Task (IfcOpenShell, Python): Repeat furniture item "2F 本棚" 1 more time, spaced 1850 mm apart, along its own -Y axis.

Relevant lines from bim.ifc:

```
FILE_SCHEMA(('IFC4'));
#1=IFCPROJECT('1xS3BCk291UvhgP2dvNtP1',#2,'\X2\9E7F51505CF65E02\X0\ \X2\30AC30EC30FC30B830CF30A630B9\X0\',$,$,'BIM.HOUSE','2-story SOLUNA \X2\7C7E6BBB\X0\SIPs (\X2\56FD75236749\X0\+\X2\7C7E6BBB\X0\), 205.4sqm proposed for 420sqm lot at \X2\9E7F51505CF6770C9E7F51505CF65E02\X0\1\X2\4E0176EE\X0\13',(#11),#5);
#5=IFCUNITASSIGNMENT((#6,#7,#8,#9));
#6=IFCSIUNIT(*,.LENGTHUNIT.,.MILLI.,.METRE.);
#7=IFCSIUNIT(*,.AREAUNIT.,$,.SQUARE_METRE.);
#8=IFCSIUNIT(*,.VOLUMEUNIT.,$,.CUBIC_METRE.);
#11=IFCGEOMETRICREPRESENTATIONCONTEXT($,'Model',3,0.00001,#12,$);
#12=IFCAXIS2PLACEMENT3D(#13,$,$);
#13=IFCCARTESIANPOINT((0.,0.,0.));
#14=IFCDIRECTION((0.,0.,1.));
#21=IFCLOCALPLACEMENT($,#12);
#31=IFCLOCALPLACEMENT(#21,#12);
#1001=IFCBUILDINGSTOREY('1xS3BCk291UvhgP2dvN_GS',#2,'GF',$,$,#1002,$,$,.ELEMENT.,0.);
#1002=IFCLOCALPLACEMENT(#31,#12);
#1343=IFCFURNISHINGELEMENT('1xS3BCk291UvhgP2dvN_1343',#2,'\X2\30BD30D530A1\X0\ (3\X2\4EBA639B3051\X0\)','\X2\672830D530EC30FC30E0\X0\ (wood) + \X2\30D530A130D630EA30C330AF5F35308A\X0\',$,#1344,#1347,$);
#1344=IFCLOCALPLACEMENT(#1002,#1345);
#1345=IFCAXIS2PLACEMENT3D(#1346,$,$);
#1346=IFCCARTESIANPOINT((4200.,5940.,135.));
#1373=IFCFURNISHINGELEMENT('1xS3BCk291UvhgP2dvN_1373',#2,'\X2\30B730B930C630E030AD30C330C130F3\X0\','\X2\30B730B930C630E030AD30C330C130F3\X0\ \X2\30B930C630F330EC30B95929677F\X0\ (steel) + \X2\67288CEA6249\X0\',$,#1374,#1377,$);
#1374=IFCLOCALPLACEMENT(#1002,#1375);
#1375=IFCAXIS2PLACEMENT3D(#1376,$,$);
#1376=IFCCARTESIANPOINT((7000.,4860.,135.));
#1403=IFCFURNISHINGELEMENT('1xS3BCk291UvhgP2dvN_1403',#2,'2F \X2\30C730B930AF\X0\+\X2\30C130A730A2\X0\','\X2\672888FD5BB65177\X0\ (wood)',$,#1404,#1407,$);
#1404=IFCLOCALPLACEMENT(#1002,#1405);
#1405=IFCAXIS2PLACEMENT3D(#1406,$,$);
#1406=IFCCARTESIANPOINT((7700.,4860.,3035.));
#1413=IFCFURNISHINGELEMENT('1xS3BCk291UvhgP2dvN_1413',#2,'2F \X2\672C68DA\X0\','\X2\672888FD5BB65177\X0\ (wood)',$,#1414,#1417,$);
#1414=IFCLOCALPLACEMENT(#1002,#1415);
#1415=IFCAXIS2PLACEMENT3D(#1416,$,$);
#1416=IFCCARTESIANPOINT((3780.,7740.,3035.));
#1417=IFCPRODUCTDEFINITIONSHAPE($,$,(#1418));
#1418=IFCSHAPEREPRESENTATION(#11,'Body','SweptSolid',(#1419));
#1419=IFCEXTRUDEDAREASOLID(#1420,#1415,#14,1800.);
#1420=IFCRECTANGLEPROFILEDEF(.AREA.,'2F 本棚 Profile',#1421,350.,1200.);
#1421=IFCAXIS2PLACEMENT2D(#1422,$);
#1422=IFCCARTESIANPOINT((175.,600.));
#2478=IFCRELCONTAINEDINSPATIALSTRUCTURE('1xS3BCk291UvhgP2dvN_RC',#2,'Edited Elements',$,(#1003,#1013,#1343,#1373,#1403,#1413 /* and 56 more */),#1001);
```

```python
import ifcopenshell
import ifcopenshell.api.geometry
import ifcopenshell.api.root
import ifcopenshell.util.element
import ifcopenshell.util.placement

model = ifcopenshell.open("bim.ifc")


def reuse_history(source, copy):
    """copy_class also copies each property set's owner history, people and application; keep the originals."""
    for rel in copy.IsDefinedBy:
        if rel.is_a("IfcRelDefinesByProperties") and (history := rel.RelatingPropertyDefinition.OwnerHistory):
            rel.RelatingPropertyDefinition.OwnerHistory = source.OwnerHistory
            ifcopenshell.util.element.remove_deep2(model, history)


source = model.by_guid("1xS3BCk291UvhgP2dvN_1413")
base = ifcopenshell.util.placement.get_local_placement(source.ObjectPlacement)
step = -base[:3, 1] * 1850.0

for i in range(1, 2):
    copy = ifcopenshell.api.root.copy_class(model, product=source)
    copy.Representation = ifcopenshell.util.element.copy_deep(
        model, source.Representation, exclude=["IfcGeometricRepresentationContext", "IfcRepresentationMap"]
    )
    reuse_history(source, copy)
    matrix = base.copy()
    matrix[:3, 3] += i * step
    print("added at", matrix[:3, 3].round(3) + 0.0)
    ifcopenshell.api.geometry.edit_object_placement(model, product=copy, matrix=matrix, is_si=False)

model.write("bim_updated.ifc")
```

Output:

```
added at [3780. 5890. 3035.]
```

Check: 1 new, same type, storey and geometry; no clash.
